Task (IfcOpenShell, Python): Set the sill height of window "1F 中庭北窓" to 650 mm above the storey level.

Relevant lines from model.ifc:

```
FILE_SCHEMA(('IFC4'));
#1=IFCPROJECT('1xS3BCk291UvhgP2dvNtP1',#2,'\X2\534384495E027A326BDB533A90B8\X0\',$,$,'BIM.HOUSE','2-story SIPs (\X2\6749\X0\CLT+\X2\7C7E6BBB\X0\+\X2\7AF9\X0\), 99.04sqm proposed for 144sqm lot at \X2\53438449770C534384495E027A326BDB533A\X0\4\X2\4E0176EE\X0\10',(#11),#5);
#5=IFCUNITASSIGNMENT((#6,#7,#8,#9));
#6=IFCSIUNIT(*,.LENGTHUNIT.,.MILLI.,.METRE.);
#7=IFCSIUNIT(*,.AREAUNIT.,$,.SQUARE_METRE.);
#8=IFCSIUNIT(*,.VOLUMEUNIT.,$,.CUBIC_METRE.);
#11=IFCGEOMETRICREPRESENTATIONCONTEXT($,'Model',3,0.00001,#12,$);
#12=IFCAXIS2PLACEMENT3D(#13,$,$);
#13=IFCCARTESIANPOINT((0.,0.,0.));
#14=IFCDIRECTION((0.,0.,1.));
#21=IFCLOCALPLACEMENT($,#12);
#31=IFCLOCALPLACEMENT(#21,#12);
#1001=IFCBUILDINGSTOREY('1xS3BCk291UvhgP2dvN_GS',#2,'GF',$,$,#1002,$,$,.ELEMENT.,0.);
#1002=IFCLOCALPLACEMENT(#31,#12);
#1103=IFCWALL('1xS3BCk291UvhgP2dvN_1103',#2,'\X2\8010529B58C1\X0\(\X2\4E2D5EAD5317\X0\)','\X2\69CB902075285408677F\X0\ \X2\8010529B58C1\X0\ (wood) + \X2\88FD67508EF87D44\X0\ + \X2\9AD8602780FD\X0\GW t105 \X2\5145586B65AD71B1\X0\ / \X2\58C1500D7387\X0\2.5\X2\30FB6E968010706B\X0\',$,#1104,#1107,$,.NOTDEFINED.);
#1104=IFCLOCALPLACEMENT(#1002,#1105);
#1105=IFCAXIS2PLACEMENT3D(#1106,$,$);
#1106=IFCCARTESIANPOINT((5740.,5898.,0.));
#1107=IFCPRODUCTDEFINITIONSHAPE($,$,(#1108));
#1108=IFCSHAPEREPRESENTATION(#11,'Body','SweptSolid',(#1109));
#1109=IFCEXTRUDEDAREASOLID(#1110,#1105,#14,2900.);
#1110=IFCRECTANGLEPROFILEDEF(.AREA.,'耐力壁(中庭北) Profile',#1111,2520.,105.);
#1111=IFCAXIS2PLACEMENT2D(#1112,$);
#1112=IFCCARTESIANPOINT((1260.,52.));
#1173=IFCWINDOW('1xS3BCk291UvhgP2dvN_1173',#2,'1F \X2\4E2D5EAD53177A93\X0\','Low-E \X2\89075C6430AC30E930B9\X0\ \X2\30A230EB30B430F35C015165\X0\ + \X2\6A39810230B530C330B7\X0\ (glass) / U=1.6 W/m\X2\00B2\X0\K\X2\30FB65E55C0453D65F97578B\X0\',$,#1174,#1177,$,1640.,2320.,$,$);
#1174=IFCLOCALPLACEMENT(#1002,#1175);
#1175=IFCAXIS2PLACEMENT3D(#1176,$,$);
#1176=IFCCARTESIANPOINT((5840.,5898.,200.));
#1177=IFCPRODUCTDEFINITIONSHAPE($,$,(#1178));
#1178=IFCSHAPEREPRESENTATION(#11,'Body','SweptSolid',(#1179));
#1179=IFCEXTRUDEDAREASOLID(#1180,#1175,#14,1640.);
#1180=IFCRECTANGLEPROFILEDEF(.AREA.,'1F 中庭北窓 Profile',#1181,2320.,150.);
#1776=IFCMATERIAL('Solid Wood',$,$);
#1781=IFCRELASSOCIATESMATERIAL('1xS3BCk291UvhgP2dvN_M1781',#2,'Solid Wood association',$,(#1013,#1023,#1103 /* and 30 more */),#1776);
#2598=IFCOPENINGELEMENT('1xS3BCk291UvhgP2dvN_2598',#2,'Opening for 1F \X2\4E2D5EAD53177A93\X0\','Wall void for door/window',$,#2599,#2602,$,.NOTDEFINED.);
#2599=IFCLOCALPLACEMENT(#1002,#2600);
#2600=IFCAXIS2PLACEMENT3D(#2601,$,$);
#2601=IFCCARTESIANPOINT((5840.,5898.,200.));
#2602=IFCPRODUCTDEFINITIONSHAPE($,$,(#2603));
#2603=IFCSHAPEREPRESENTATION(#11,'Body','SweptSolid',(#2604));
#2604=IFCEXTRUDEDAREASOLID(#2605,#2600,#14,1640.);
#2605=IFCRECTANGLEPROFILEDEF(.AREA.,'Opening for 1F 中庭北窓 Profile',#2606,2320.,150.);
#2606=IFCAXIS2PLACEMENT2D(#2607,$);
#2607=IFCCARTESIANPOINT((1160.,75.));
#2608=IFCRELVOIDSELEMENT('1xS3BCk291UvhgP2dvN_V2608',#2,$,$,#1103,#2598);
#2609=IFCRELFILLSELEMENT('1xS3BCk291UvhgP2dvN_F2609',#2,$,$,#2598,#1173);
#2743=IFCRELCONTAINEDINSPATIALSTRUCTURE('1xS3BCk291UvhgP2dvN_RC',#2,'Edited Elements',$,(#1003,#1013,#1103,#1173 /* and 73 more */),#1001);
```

```python
import numpy as np
import ifcopenshell
import ifcopenshell.api.geometry
import ifcopenshell.geom
import ifcopenshell.util.element
import ifcopenshell.util.placement
import ifcopenshell.util.shape
import ifcopenshell.util.unit

model = ifcopenshell.open("model.ifc")
unit_scale = ifcopenshell.util.unit.calculate_unit_scale(model)

window = model.by_id(1173)
opening = window.FillsVoids[0].RelatingOpeningElement
storey = ifcopenshell.util.element.get_container(window, ifc_class="IfcBuildingStorey")
level = ifcopenshell.util.placement.get_local_placement(storey.ObjectPlacement)[2, 3]

# The opening's origin need not be at the sill, so measure its lowest point.
shape = ifcopenshell.geom.create_shape(ifcopenshell.geom.settings(), opening)
bottom = ifcopenshell.util.shape.get_shape_bottom_elevation(shape, shape.geometry) / unit_scale
dz = level + 0.65 / unit_scale - bottom

shift = np.array([0.0, 0.0, dz])
# The window is not placed relative to its opening, so move both.
for product in (opening, window):
    matrix = ifcopenshell.util.placement.get_local_placement(product.ObjectPlacement)
    matrix[:3, 3] += shift
    ifcopenshell.api.geometry.edit_object_placement(model, product=product, matrix=matrix, is_si=False)

print(f"moved by {dz * unit_scale:+.3f} m")

model.write("model_edited.ifc")
```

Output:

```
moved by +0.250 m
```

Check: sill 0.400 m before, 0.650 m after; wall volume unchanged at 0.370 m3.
